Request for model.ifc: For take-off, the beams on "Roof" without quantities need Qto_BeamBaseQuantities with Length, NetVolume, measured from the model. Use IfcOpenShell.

First a look at what the model holds.

```python
import ifcopenshell
import ifcopenshell.util.element
import ifcopenshell.util.unit

model = ifcopenshell.open("model.ifc")
print(model.schema)
for unit_type in ("LENGTHUNIT", "AREAUNIT", "VOLUMEUNIT"):
    print(unit_type, ifcopenshell.util.unit.calculate_unit_scale(model, unit_type))
storey = next(s for s in model.by_type("IfcBuildingStorey") if s.Name == "Roof")
beams = [e for e in ifcopenshell.util.element.get_decomposition(storey) if e.is_a("IfcBeam")]
for e in sorted(beams, key=lambda e: e.id()):
    print(e.id(), e.is_a(), e.Name, list(ifcopenshell.util.element.get_psets(e, qtos_only=True)), sep=" | ")
```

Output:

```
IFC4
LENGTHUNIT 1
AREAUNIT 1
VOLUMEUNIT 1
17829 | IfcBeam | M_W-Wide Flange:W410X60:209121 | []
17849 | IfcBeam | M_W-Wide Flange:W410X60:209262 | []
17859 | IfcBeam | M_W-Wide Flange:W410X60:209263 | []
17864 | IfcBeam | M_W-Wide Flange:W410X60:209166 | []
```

```python
import ifcopenshell
import ifcopenshell.api.pset
import ifcopenshell.geom
import ifcopenshell.util.element
import ifcopenshell.util.shape
import ifcopenshell.util.unit

model = ifcopenshell.open("model.ifc")
unit_scale = ifcopenshell.util.unit.calculate_unit_scale(model)
volume_scale = ifcopenshell.util.unit.calculate_unit_scale(model, "VOLUMEUNIT")
settings = ifcopenshell.geom.settings()

storey = next(s for s in model.by_type("IfcBuildingStorey") if s.Name == "Roof")
beams = [e for e in ifcopenshell.util.element.get_decomposition(storey) if e.is_a("IfcBeam")]

for e in sorted(beams, key=lambda e: e.id()):
    if ifcopenshell.util.element.get_psets(e, qtos_only=True, should_inherit=False):
        continue
    # Geometry comes back in metres, in the element's own axes.
    shape = ifcopenshell.geom.create_shape(settings, e)
    values = {
        "Length": ifcopenshell.util.shape.get_max_xyz(shape.geometry) / unit_scale,
        "NetVolume": ifcopenshell.util.shape.get_volume(shape.geometry) / volume_scale,
    }
    qto = ifcopenshell.api.pset.add_qto(model, product=e, name="Qto_BeamBaseQuantities")
    ifcopenshell.api.pset.edit_qto(model, qto=qto, properties=values)
    print(e.id(), {k: round(v, 3) for k, v in values.items()})

model.write("model_v2.ifc")
```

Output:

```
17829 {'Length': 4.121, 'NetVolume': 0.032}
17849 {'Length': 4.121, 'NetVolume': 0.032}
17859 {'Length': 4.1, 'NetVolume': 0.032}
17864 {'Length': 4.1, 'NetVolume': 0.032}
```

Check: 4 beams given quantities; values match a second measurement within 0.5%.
